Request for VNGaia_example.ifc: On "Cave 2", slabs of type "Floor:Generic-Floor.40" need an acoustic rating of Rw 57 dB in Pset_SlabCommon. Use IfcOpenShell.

First a look at what the model holds.

```python
import ifcopenshell
import ifcopenshell.util.element

model = ifcopenshell.open("VNGaia_example.ifc")
print(model.schema)
storey = next(s for s in model.by_type("IfcBuildingStorey") if s.Name == "Cave 2")
slabs = [e for e in ifcopenshell.util.element.get_decomposition(storey) if e.is_a("IfcSlab")]
seen = {}
for e in slabs:
    element_type = ifcopenshell.util.element.get_type(e)
    key = (element_type.Name if element_type != e and element_type else None, ifcopenshell.util.element.get_pset(e, "Pset_SlabCommon", "AcousticRating"))
    seen[key] = seen.get(key, 0) + 1
for (name, value), count in sorted(seen.items(), key=str):
    print(count, "x", name, "|", value)
```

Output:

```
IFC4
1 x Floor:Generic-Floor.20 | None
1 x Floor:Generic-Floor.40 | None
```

```python
import ifcopenshell
import ifcopenshell.api.pset
import ifcopenshell.util.element

model = ifcopenshell.open("VNGaia_example.ifc")

storey = next(s for s in model.by_type("IfcBuildingStorey") if s.Name == "Cave 2")
slabs = [e for e in ifcopenshell.util.element.get_decomposition(storey) if e.is_a("IfcSlab")]

count = 0
for e in slabs:
    element_type = ifcopenshell.util.element.get_type(e)
    if element_type in (None, e) or element_type.Name != "Floor:Generic-Floor.40":
        continue
    # add_pset returns the element's existing set when there is one.
    pset = ifcopenshell.api.pset.add_pset(model, product=e, name="Pset_SlabCommon")
    ifcopenshell.api.pset.edit_pset(model, pset=pset, properties={"AcousticRating": "Rw 57 dB"})
    count += 1

print(count, "slabs updated")

model.write("VNGaia_example_v2.ifc")
```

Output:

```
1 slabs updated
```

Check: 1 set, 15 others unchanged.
